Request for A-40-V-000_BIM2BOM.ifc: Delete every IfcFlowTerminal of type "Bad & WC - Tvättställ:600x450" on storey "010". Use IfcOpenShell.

First a look at what the model holds.

```python
import ifcopenshell
import ifcopenshell.util.element

model = ifcopenshell.open("A-40-V-000_BIM2BOM.ifc")
print(model.schema)
storey = next(s for s in model.by_type("IfcBuildingStorey") if s.Name == "010")
terminals = [e for e in ifcopenshell.util.element.get_decomposition(storey) if e.is_a("IfcFlowTerminal")]
seen = {}
for e in terminals:
    element_type = ifcopenshell.util.element.get_type(e)
    name = element_type.Name if element_type not in (None, e) else None
    seen[name] = seen.get(name, 0) + 1
for name, count in sorted(seen.items(), key=str):
    print(count, "x", name)
```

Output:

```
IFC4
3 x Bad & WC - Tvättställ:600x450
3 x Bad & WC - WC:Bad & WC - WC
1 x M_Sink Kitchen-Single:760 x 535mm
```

```python
import ifcopenshell
import ifcopenshell.api.root
import ifcopenshell.util.element

model = ifcopenshell.open("A-40-V-000_BIM2BOM.ifc")

storey = next(s for s in model.by_type("IfcBuildingStorey") if s.Name == "010")
terminals = [e for e in ifcopenshell.util.element.get_decomposition(storey) if e.is_a("IfcFlowTerminal")]
targets = [e for e in terminals if (t := ifcopenshell.util.element.get_type(e)) not in (None, e) and t.Name == "Bad & WC - Tvättställ:600x450"]

for e in targets:
    ifcopenshell.api.root.remove_product(model, product=e)
print(len(targets), "removed")

model.write("A-40-V-000_BIM2BOM_updated.ifc")
```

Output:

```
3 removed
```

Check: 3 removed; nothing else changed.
